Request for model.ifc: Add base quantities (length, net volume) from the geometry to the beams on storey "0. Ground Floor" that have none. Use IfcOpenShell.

First a look at what the model holds.

```python
import ifcopenshell
import ifcopenshell.util.element
import ifcopenshell.util.unit

model = ifcopenshell.open("model.ifc")
print(model.schema)
for unit_type in ("LENGTHUNIT", "AREAUNIT", "VOLUMEUNIT"):
    print(unit_type, ifcopenshell.util.unit.calculate_unit_scale(model, unit_type))
storey = next(s for s in model.by_type("IfcBuildingStorey") if s.Name == "0. Ground Floor")
beams = [e for e in ifcopenshell.util.element.get_decomposition(storey) if e.is_a("IfcBeam")]
for e in sorted(beams, key=lambda e: e.id()):
    print(e.id(), e.is_a(), e.Name, list(ifcopenshell.util.element.get_psets(e, qtos_only=True)), sep=" | ")
```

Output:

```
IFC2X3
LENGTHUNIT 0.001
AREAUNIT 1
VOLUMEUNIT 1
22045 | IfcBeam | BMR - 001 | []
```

```python
import ifcopenshell
import ifcopenshell.api.pset
import ifcopenshell.geom
import ifcopenshell.util.element
import ifcopenshell.util.shape
import ifcopenshell.util.unit

model = ifcopenshell.open("model.ifc")
unit_scale = ifcopenshell.util.unit.calculate_unit_scale(model)
volume_scale = ifcopenshell.util.unit.calculate_unit_scale(model, "VOLUMEUNIT")
settings = ifcopenshell.geom.settings()

storey = next(s for s in model.by_type("IfcBuildingStorey") if s.Name == "0. Ground Floor")
beams = [e for e in ifcopenshell.util.element.get_decomposition(storey) if e.is_a("IfcBeam")]

for e in sorted(beams, key=lambda e: e.id()):
    if ifcopenshell.util.element.get_psets(e, qtos_only=True, should_inherit=False):
        continue
    # Geometry comes back in metres, in the element's own axes.
    shape = ifcopenshell.geom.create_shape(settings, e)
    values = {
        "Length": ifcopenshell.util.shape.get_max_xyz(shape.geometry) / unit_scale,
        "NetVolume": ifcopenshell.util.shape.get_volume(shape.geometry) / volume_scale,
    }
    qto = ifcopenshell.api.pset.add_qto(model, product=e, name="BaseQuantities")
    ifcopenshell.api.pset.edit_qto(model, qto=qto, properties=values)
    print(e.id(), {k: round(v, 3) for k, v in values.items()})

model.write("model_edited.ifc")
```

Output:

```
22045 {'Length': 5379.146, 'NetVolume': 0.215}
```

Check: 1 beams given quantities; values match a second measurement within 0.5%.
